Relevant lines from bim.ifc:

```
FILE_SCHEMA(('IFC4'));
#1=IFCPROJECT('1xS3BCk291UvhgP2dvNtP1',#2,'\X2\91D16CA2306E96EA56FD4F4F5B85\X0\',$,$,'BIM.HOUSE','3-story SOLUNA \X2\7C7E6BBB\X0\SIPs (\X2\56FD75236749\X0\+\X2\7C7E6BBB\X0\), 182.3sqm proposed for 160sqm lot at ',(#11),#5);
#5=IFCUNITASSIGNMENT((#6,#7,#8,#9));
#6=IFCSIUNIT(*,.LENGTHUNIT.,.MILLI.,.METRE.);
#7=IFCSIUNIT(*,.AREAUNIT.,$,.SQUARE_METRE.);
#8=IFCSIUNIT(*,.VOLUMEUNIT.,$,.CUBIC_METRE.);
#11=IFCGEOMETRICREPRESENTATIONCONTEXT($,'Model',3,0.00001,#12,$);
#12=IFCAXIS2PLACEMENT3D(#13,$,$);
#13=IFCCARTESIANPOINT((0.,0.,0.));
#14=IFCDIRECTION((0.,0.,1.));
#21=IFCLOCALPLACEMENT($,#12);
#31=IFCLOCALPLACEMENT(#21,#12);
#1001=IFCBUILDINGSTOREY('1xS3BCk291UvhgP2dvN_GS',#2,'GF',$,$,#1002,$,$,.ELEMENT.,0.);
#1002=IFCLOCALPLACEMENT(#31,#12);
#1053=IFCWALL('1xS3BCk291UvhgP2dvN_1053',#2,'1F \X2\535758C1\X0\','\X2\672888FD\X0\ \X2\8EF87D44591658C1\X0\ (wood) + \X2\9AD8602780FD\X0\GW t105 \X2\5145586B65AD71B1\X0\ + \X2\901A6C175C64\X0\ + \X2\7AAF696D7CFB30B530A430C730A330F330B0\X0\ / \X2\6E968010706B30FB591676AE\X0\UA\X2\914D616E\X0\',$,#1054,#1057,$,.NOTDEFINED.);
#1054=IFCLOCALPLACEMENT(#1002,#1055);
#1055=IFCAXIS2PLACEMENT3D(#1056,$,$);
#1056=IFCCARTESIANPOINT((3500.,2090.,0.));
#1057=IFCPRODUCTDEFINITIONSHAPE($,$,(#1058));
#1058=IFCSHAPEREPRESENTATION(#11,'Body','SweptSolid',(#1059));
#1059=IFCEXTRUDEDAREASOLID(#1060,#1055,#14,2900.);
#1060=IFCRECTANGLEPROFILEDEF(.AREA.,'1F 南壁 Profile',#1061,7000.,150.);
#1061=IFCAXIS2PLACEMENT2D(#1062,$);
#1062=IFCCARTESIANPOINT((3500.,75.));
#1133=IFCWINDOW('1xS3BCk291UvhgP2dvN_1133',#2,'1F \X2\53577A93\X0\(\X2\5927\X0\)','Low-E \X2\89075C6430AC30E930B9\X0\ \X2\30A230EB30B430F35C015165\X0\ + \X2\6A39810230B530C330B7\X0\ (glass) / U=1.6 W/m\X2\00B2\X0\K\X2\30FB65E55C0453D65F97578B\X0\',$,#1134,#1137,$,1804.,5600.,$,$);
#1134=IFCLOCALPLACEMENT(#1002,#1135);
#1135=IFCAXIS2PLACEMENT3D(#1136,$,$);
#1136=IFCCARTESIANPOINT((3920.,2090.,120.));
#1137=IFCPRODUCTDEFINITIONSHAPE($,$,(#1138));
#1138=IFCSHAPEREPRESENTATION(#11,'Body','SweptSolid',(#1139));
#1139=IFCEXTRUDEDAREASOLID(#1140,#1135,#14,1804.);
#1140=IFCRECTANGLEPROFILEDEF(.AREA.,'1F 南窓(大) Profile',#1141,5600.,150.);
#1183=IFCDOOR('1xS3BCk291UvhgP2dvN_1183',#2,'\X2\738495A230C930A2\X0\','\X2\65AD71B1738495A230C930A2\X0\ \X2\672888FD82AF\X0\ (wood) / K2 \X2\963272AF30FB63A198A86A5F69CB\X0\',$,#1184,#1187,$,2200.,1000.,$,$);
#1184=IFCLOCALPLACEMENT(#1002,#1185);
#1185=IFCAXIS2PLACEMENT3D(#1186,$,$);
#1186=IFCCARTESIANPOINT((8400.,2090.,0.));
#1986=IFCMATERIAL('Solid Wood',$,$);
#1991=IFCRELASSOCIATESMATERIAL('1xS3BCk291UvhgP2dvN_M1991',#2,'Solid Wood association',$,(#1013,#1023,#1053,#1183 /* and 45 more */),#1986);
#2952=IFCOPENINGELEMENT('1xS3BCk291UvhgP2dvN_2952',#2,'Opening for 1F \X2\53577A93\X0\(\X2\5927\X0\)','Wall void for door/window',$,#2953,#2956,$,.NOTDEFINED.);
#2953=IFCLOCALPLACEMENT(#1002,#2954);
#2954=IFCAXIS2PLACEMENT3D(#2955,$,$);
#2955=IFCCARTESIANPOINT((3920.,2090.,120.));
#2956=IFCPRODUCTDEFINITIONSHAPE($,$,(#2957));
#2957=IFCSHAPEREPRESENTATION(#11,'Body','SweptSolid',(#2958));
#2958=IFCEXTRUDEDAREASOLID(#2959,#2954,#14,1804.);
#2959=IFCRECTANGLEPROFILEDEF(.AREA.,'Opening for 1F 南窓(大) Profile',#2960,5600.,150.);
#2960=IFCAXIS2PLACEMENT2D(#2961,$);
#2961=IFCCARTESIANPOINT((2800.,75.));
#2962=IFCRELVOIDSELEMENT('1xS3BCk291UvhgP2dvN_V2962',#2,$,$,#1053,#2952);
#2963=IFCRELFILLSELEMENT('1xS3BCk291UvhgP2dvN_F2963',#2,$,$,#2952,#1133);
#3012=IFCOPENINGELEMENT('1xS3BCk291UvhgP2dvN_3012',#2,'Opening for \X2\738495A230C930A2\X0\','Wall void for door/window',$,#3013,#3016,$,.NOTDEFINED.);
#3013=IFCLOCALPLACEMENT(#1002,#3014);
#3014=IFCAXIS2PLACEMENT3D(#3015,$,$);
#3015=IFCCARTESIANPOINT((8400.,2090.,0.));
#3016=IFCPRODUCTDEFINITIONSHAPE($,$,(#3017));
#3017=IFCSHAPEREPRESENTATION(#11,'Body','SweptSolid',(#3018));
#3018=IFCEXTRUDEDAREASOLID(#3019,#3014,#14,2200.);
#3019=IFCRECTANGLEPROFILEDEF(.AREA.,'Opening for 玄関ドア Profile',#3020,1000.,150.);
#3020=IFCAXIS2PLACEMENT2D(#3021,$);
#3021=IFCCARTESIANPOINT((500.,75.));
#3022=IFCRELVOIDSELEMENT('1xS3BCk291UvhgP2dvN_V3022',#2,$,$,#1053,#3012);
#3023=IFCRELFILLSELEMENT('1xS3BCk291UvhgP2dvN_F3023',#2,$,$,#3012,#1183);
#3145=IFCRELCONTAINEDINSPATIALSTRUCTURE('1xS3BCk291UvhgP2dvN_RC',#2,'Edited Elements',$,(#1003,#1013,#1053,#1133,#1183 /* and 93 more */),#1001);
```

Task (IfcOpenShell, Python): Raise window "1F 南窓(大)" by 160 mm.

```python
import numpy as np
import ifcopenshell
import ifcopenshell.api.geometry
import ifcopenshell.util.placement
import ifcopenshell.util.unit

model = ifcopenshell.open("bim.ifc")
unit_scale = ifcopenshell.util.unit.calculate_unit_scale(model)

window = model.by_id(1133)
opening = window.FillsVoids[0].RelatingOpeningElement
dz = 0.16 / unit_scale

shift = np.array([0.0, 0.0, dz])
# The window is not placed relative to its opening, so move both.
for product in (opening, window):
    matrix = ifcopenshell.util.placement.get_local_placement(product.ObjectPlacement)
    matrix[:3, 3] += shift
    ifcopenshell.api.geometry.edit_object_placement(model, product=product, matrix=matrix, is_si=False)

print(f"moved by {dz * unit_scale:+.3f} m")

model.write("bim_v2.ifc")
```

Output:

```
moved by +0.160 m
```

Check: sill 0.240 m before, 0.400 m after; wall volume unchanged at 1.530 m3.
